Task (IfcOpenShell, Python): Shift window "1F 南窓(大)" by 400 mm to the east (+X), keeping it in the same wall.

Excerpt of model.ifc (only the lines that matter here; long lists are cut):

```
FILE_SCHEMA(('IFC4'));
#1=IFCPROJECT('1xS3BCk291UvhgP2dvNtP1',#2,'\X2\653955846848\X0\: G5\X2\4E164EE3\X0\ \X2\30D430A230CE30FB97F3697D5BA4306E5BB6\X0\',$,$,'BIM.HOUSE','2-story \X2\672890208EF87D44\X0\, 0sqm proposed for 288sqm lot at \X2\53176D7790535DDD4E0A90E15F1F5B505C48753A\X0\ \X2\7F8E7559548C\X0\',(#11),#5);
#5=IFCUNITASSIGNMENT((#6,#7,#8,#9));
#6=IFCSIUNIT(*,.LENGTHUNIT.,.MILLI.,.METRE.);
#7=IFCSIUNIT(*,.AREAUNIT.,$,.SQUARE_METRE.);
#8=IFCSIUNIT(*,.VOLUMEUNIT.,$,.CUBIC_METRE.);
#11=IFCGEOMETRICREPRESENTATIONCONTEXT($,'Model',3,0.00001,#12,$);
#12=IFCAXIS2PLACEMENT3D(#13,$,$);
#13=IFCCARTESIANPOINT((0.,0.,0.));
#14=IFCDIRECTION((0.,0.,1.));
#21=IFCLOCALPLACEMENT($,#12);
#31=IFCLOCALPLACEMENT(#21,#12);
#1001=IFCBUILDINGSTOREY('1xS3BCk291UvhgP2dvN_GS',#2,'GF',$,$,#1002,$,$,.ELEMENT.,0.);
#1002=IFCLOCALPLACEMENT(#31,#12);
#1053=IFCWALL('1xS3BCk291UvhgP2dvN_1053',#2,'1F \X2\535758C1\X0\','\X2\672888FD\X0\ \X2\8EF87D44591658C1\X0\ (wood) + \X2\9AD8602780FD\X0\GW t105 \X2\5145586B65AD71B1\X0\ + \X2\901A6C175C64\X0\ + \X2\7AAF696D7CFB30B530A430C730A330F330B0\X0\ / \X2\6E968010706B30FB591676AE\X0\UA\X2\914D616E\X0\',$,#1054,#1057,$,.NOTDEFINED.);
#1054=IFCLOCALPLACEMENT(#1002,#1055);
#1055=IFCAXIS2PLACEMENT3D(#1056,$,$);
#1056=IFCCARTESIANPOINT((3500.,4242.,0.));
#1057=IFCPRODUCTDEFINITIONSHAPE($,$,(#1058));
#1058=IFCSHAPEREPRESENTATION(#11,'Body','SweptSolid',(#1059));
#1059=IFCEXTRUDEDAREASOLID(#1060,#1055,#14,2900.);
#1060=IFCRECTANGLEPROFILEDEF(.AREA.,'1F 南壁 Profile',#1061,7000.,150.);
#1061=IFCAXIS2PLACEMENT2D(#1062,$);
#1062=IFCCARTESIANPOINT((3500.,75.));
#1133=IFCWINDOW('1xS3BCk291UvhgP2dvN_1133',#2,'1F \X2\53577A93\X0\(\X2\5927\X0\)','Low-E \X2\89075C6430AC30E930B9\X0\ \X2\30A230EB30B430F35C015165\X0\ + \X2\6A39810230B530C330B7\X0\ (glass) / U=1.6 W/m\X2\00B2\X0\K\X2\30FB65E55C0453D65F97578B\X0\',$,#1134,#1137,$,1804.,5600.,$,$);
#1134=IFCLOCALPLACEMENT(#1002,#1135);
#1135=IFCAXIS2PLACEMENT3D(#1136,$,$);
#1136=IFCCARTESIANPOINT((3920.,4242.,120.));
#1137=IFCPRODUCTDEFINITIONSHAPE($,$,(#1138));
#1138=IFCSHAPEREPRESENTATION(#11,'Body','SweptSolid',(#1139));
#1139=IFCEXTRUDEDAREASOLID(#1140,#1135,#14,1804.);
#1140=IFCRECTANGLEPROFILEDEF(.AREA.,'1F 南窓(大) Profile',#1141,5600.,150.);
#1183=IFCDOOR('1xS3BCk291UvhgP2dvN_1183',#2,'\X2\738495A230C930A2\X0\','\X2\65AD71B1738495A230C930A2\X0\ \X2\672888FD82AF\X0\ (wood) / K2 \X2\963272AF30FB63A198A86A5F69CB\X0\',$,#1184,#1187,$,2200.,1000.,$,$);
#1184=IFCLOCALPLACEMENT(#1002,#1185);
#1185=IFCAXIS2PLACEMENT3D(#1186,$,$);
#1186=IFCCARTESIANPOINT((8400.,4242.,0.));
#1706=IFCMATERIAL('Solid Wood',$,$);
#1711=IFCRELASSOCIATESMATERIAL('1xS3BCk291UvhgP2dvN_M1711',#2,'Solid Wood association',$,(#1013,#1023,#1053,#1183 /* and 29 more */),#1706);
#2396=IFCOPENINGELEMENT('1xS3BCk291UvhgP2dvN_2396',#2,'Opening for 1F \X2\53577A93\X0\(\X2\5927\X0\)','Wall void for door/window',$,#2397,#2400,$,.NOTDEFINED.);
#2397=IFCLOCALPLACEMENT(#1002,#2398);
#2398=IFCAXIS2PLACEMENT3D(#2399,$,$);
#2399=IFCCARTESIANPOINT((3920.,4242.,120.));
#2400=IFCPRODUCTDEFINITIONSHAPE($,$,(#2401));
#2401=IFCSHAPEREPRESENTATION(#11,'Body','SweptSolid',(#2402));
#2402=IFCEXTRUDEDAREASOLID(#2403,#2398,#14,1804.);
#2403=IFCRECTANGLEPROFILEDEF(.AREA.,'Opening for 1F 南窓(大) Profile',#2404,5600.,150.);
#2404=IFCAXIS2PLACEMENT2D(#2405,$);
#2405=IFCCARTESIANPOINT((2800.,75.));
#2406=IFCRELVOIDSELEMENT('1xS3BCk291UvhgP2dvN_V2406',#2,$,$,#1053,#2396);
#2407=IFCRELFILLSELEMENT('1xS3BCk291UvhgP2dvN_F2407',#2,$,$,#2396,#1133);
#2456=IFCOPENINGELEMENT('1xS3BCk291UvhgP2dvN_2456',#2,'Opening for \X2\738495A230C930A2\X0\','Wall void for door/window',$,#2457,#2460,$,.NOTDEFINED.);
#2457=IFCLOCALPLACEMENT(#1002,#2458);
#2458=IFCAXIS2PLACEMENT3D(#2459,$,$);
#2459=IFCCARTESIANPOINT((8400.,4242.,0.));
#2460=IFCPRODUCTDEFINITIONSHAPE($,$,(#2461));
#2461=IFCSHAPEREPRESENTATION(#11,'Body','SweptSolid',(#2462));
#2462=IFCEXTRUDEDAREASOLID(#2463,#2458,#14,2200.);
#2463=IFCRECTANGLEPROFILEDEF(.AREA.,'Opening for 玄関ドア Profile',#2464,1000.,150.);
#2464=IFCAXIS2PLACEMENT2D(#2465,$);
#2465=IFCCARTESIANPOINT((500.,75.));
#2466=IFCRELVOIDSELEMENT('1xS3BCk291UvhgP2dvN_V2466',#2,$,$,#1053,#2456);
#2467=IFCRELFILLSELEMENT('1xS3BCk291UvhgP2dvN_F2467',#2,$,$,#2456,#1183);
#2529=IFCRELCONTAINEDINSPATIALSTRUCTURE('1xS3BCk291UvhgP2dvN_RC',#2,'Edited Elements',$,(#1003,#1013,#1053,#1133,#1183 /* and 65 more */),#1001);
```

```python
import ifcopenshell
import ifcopenshell.api.geometry
import ifcopenshell.util.placement
import ifcopenshell.util.unit

model = ifcopenshell.open("model.ifc")
unit_scale = ifcopenshell.util.unit.calculate_unit_scale(model)

window = model.by_id(1133)
opening = window.FillsVoids[0].RelatingOpeningElement
wall = opening.VoidsElements[0].RelatingBuildingElement

wall_matrix = ifcopenshell.util.placement.get_local_placement(wall.ObjectPlacement)
shift = wall_matrix[:3, 0] * 0.4 / unit_scale
before = ifcopenshell.util.placement.get_local_placement(window.ObjectPlacement)[:3, 3].copy()

# The window is not placed relative to its opening, so move both.
for product in (opening, window):
    matrix = ifcopenshell.util.placement.get_local_placement(product.ObjectPlacement)
    matrix[:3, 3] += shift
    ifcopenshell.api.geometry.edit_object_placement(model, product=product, matrix=matrix, is_si=False)

after = ifcopenshell.util.placement.get_local_placement(window.ObjectPlacement)[:3, 3]
print("window moved by", (after - before).round(3) + 0.0)

model.write("model_rev.ifc")
```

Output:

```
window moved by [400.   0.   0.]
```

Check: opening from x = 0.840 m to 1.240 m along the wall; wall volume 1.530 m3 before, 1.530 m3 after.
